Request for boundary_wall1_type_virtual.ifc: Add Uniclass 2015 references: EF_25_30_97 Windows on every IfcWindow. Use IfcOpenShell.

First a look at what the model holds.

```python
import ifcopenshell

model = ifcopenshell.open("boundary_wall1_type_virtual.ifc")
print(model.schema)
print("classifications:", [c.Name for c in model.by_type("IfcClassification")])
for ifc_class in ("IfcDoor", "IfcRoof", "IfcStair", "IfcWall", "IfcWindow"):
    print(ifc_class, len(model.by_type(ifc_class)))
```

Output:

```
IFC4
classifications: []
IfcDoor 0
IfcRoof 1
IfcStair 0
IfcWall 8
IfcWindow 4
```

```python
import ifcopenshell
import ifcopenshell.api.classification

model = ifcopenshell.open("boundary_wall1_type_virtual.ifc")

system = ifcopenshell.api.classification.add_classification(model, classification="Uniclass 2015")

codes = {
    "IfcWindow": ("EF_25_30_97", "Windows"),
}
for ifc_class, (code, name) in codes.items():
    products = model.by_type(ifc_class)
    ifcopenshell.api.classification.add_reference(
        model, products=products, classification=system, identification=code, name=name
    )
    print(code, len(products))

model.write("boundary_wall1_type_virtual_rev.ifc")
```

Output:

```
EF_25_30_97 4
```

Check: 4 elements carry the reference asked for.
